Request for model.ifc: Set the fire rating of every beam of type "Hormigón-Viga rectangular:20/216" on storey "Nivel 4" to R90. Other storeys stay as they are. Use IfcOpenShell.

First a look at what the model holds.

```python
import ifcopenshell
import ifcopenshell.util.element

model = ifcopenshell.open("model.ifc")
print(model.schema)
storey = next(s for s in model.by_type("IfcBuildingStorey") if s.Name == "Nivel 4")
beams = [e for e in ifcopenshell.util.element.get_decomposition(storey) if e.is_a("IfcBeam")]
seen = {}
for e in beams:
    element_type = ifcopenshell.util.element.get_type(e)
    key = (element_type.Name if element_type != e and element_type else None, ifcopenshell.util.element.get_pset(e, "Pset_BeamCommon", "FireRating"))
    seen[key] = seen.get(key, 0) + 1
for (name, value), count in sorted(seen.items(), key=str):
    print(count, "x", name, "|", value)
```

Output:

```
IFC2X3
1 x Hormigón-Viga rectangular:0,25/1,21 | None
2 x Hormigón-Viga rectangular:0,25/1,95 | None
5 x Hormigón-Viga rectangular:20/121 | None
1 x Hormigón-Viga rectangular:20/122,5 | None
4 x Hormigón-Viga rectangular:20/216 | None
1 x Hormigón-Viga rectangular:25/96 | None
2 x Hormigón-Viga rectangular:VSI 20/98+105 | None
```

```python
import ifcopenshell
import ifcopenshell.api.pset
import ifcopenshell.util.element

model = ifcopenshell.open("model.ifc")

storey = next(s for s in model.by_type("IfcBuildingStorey") if s.Name == "Nivel 4")
beams = [e for e in ifcopenshell.util.element.get_decomposition(storey) if e.is_a("IfcBeam")]

count = 0
for e in beams:
    element_type = ifcopenshell.util.element.get_type(e)
    if element_type in (None, e) or element_type.Name != "Hormigón-Viga rectangular:20/216":
        continue
    # add_pset returns the element's existing set when there is one.
    pset = ifcopenshell.api.pset.add_pset(model, product=e, name="Pset_BeamCommon")
    ifcopenshell.api.pset.edit_pset(model, pset=pset, properties={"FireRating": "R90"})
    count += 1

print(count, "beams updated")

model.write("model-out.ifc")
```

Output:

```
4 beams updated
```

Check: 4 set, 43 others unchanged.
